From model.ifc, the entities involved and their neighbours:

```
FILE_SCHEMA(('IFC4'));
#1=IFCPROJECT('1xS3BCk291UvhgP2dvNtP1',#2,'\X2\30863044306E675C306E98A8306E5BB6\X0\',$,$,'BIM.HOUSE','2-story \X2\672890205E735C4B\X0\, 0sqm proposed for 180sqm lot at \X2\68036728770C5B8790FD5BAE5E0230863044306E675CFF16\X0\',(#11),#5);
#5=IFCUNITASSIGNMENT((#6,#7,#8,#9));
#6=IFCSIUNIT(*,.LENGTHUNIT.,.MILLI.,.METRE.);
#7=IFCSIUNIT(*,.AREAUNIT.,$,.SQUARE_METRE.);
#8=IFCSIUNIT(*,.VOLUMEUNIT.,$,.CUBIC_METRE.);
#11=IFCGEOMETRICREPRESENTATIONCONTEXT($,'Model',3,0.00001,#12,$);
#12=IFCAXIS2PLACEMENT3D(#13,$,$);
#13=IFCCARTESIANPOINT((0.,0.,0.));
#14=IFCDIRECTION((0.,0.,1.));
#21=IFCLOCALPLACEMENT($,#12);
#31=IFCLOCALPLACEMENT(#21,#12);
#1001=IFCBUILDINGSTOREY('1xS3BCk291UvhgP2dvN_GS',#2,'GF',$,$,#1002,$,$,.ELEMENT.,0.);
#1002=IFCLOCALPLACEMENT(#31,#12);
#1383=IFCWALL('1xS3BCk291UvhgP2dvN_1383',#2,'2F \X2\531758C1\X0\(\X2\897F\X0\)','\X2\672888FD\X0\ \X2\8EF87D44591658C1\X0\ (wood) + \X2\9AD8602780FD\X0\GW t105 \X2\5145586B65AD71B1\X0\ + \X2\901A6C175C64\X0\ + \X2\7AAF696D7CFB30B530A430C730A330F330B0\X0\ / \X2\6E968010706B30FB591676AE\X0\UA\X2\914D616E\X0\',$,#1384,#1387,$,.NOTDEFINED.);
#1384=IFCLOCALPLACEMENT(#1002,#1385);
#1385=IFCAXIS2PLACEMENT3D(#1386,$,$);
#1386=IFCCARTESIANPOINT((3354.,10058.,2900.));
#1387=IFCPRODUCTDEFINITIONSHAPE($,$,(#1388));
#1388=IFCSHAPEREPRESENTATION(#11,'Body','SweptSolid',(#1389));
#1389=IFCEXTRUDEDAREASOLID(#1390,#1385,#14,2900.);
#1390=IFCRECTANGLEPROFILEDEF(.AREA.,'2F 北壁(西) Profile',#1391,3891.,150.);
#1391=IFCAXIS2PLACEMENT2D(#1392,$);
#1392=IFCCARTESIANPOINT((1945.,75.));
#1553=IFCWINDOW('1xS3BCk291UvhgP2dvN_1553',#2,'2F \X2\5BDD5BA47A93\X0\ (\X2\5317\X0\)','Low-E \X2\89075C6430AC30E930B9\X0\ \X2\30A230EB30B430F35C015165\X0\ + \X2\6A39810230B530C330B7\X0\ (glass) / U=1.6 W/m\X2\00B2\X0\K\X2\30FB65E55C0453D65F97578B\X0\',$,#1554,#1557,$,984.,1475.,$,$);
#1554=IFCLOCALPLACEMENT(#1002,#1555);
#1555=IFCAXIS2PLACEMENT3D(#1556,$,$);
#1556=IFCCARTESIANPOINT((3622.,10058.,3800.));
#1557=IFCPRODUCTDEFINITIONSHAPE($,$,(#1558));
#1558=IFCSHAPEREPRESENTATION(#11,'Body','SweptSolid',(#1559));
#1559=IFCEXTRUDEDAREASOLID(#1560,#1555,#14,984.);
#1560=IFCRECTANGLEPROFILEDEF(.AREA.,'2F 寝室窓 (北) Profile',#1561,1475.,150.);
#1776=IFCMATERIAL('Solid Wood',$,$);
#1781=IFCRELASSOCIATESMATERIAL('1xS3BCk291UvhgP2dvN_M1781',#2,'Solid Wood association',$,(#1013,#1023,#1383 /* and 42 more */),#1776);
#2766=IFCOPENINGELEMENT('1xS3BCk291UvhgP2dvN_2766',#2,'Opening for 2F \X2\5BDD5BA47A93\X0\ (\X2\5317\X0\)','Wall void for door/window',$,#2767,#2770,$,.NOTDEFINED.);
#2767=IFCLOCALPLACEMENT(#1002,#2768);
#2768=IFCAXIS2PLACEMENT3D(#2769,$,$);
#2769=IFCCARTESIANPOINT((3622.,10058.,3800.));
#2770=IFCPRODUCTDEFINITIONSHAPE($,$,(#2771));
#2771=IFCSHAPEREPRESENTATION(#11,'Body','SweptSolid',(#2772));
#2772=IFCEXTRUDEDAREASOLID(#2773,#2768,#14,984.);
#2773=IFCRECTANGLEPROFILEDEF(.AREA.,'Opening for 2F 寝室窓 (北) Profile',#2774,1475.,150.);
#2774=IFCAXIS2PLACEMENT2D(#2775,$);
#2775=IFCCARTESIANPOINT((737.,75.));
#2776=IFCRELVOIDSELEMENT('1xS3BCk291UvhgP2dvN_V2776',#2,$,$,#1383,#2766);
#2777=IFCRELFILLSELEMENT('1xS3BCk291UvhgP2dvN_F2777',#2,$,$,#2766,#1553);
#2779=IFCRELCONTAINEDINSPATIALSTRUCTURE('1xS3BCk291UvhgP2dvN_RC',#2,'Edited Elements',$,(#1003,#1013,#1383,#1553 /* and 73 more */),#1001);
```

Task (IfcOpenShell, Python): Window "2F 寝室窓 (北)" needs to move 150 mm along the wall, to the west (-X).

```python
import ifcopenshell
import ifcopenshell.api.geometry
import ifcopenshell.util.placement

model = ifcopenshell.open("model.ifc")

window = model.by_guid("1xS3BCk291UvhgP2dvN_1553")
opening = window.FillsVoids[0].RelatingOpeningElement
wall = opening.VoidsElements[0].RelatingBuildingElement

wall_matrix = ifcopenshell.util.placement.get_local_placement(wall.ObjectPlacement)
shift = wall_matrix[:3, 0] * -150.0
before = ifcopenshell.util.placement.get_local_placement(window.ObjectPlacement)[:3, 3].copy()

# The window is not placed relative to its opening, so move both.
for product in (opening, window):
    matrix = ifcopenshell.util.placement.get_local_placement(product.ObjectPlacement)
    matrix[:3, 3] += shift
    ifcopenshell.api.geometry.edit_object_placement(model, product=product, matrix=matrix, is_si=False)

after = ifcopenshell.util.placement.get_local_placement(window.ObjectPlacement)[:3, 3]
print("window moved by", (after - before).round(3) + 0.0)

model.write("model-out.ifc")
```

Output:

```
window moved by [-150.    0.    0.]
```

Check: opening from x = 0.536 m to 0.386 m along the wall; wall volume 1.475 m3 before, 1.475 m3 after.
